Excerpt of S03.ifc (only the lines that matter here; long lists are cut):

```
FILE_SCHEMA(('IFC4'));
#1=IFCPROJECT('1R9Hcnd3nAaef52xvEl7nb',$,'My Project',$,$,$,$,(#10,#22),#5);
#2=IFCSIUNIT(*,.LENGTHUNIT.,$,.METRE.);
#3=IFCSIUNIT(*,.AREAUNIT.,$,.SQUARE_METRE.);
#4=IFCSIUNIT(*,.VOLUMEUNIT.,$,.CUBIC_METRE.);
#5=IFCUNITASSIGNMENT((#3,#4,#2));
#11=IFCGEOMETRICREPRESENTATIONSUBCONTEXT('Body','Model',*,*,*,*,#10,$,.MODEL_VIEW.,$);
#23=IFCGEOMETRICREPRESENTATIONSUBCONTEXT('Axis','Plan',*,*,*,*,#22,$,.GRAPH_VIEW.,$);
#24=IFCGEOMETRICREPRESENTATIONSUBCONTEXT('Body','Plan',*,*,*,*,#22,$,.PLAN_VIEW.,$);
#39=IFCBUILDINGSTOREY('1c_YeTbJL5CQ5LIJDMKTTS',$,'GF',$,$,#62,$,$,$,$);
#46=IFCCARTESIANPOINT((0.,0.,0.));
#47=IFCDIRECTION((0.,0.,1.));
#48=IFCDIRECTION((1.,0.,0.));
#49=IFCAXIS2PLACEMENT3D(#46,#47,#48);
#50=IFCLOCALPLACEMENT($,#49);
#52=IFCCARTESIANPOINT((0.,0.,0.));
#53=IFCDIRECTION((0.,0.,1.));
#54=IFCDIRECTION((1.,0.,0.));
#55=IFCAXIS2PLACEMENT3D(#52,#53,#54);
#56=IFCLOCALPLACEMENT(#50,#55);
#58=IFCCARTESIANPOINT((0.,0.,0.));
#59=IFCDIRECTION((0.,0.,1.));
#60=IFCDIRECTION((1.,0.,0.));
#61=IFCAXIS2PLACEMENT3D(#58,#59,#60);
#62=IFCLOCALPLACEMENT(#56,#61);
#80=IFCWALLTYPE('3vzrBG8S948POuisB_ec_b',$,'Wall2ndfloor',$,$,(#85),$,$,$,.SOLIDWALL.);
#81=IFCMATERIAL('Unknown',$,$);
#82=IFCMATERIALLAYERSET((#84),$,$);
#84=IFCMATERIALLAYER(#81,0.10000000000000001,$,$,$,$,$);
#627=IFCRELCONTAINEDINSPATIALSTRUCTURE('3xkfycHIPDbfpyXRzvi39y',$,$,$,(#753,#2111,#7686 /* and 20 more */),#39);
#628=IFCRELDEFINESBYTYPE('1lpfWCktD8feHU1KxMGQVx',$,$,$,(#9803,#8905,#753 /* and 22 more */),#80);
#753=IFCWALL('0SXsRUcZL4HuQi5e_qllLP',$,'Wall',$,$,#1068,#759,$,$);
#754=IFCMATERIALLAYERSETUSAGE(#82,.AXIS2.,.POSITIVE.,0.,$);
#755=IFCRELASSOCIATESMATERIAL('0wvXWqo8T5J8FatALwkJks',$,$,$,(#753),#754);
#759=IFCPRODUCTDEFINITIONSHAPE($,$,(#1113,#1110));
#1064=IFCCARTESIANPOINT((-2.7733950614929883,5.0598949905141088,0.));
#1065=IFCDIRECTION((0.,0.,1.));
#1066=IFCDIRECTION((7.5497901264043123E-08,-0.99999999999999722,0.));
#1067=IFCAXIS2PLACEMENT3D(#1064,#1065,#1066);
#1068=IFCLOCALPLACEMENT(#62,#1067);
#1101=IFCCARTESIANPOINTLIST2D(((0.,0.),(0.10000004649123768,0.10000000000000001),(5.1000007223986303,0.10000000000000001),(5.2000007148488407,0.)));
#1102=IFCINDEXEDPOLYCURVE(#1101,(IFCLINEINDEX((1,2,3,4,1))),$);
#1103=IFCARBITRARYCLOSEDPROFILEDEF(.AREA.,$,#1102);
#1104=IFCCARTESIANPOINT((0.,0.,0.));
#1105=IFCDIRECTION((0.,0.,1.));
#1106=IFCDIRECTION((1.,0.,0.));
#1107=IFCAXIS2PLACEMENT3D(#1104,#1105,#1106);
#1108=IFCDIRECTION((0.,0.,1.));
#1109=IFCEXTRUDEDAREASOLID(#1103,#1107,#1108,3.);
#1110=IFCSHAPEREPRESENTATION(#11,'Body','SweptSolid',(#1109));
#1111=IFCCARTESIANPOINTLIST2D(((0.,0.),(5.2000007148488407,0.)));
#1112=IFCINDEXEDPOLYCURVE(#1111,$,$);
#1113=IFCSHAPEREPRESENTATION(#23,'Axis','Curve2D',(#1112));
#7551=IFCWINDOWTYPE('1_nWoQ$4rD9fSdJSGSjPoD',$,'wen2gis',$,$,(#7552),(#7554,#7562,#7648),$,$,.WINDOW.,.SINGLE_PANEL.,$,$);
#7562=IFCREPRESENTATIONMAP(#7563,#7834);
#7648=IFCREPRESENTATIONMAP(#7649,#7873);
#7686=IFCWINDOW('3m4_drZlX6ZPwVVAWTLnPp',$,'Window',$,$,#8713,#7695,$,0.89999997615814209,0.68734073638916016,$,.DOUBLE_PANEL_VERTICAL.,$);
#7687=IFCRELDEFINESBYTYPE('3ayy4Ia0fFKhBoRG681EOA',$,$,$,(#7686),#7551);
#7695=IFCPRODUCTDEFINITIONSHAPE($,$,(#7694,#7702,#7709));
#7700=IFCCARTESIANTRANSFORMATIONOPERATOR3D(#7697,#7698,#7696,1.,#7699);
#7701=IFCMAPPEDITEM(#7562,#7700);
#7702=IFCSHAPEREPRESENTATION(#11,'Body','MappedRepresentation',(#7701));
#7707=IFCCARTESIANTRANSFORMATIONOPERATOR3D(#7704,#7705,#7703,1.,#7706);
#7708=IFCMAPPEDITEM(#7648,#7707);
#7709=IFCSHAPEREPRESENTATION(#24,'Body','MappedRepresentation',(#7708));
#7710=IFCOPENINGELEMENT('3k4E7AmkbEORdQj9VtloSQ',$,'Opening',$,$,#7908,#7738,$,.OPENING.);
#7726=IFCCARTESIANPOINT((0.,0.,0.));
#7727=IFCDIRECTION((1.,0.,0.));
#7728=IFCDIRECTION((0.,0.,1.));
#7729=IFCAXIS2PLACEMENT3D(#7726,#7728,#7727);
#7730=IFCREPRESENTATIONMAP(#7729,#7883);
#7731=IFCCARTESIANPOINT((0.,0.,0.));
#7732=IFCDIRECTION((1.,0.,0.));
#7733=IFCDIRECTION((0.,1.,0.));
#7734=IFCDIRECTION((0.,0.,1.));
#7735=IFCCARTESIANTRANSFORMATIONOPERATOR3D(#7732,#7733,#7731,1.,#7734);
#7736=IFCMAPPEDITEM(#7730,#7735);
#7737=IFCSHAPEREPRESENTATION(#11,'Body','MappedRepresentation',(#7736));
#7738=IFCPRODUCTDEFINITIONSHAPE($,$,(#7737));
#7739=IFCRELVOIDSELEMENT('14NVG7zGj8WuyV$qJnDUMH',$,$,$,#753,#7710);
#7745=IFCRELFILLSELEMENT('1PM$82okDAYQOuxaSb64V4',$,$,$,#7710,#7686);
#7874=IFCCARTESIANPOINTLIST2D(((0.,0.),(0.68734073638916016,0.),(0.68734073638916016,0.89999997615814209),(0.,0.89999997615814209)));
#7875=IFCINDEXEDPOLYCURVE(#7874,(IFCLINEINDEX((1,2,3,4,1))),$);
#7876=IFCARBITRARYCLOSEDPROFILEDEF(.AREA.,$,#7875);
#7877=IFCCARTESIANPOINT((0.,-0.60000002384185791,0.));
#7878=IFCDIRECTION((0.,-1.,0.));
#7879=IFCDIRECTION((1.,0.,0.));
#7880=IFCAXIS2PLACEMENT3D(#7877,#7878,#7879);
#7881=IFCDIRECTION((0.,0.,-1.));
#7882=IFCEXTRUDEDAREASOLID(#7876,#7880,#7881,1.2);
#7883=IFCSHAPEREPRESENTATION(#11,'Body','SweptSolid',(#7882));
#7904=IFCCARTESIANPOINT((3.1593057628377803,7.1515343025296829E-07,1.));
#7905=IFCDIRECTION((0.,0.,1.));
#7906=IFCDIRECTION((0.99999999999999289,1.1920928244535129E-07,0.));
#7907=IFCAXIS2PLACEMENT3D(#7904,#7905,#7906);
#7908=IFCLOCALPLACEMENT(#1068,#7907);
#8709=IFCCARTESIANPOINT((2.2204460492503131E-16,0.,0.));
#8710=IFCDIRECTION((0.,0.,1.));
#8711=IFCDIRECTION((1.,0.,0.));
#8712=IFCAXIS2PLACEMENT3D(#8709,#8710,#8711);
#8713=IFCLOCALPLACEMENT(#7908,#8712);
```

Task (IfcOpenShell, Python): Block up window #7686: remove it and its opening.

```python
import ifcopenshell
import ifcopenshell.api.feature
import ifcopenshell.api.root
import ifcopenshell.geom
import ifcopenshell.util.shape

model = ifcopenshell.open("S03.ifc")
settings = ifcopenshell.geom.settings()


def volume(element):
    """Net volume in cubic metres, openings subtracted."""
    shape = ifcopenshell.geom.create_shape(settings, element)
    return ifcopenshell.util.shape.get_volume(shape.geometry)


window = model.by_id(7686)
opening = window.FillsVoids[0].RelatingOpeningElement
wall = opening.VoidsElements[0].RelatingBuildingElement
before = volume(wall)

ifcopenshell.api.root.remove_product(model, product=window)
ifcopenshell.api.feature.remove_feature(model, feature=opening)

after = volume(wall)

print(f"wall volume {before:.3f} -> {after:.3f} m3")

model.write("S03_edited.ifc")
```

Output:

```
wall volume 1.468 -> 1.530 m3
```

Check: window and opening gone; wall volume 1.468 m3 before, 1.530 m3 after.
